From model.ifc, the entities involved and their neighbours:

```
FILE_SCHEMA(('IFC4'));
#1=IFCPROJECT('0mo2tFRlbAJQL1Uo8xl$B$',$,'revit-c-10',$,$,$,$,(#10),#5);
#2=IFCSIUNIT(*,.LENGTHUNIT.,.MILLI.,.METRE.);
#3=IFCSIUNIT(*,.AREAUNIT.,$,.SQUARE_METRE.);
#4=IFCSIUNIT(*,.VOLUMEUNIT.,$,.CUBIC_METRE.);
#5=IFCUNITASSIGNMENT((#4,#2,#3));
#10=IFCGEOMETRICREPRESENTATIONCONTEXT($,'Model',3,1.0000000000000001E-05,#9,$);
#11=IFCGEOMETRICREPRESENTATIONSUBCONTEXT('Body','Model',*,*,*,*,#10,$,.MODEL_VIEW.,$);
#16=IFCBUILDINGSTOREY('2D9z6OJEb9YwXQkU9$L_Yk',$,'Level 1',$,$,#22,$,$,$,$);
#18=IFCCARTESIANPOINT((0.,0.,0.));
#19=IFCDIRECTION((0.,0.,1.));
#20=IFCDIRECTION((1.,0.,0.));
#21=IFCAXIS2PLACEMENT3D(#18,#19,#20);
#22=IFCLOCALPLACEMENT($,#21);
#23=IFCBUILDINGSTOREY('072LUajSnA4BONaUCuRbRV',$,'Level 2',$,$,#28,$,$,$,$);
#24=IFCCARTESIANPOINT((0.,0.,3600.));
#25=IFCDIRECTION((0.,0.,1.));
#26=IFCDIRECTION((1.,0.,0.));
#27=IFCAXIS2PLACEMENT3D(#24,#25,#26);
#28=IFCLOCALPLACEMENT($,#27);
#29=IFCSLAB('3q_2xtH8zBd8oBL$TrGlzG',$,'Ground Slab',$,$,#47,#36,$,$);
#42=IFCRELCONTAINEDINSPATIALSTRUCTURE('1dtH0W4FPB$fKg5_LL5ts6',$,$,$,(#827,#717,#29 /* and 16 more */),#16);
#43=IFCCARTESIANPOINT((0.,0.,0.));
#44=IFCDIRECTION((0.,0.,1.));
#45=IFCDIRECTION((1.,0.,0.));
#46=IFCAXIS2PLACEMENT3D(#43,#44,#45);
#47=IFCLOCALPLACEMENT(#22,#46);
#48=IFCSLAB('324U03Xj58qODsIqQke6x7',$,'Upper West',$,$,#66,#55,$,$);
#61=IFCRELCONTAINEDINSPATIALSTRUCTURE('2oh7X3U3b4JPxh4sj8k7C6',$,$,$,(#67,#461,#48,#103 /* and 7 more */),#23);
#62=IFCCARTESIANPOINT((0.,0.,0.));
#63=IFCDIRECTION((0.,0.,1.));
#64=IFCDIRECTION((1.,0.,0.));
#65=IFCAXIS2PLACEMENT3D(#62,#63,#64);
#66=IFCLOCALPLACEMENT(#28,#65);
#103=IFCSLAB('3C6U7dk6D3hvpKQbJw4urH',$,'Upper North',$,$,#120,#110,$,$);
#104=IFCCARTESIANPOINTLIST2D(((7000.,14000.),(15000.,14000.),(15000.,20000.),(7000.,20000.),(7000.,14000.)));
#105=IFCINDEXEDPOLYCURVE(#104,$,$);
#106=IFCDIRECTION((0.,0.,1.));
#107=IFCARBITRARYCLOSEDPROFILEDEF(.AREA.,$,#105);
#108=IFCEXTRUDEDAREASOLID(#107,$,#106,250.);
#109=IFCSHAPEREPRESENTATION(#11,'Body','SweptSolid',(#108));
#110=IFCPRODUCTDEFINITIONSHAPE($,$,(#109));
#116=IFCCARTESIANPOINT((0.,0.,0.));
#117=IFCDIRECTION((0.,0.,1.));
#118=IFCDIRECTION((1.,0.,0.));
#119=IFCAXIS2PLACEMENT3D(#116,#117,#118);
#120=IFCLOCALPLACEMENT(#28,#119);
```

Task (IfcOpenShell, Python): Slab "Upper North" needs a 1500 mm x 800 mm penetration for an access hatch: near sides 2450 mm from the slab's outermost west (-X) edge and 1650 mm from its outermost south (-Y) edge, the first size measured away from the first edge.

```python
import numpy as np
import ifcopenshell
import ifcopenshell.api.feature
import ifcopenshell.api.geometry
import ifcopenshell.api.root
import ifcopenshell.geom
import ifcopenshell.util.placement
import ifcopenshell.util.representation
import ifcopenshell.util.shape
import ifcopenshell.util.unit

model = ifcopenshell.open("model.ifc")
unit_scale = ifcopenshell.util.unit.calculate_unit_scale(model)
settings = ifcopenshell.geom.settings()


def volume(element):
    """Net volume in cubic metres, openings subtracted."""
    shape = ifcopenshell.geom.create_shape(settings, element)
    return ifcopenshell.util.shape.get_volume(shape.geometry)


slab = model.by_id(103)
before = volume(slab)

# Extent in the slab's own axes, in metres. The edges named are its -X and -Y sides.
slab_shape = ifcopenshell.geom.create_shape(settings, slab)
vertices = ifcopenshell.util.shape.get_vertices(slab_shape.geometry)
x_min, y_min, bottom = vertices.min(axis=0)
top = vertices[:, 2].max()

opening = ifcopenshell.api.root.create_entity(model, ifc_class="IfcOpeningElement", name="Access hatch opening", predefined_type="OPENING")
context = ifcopenshell.util.representation.get_context(model, "Model", "Body", "MODEL_VIEW")
width, depth = 1.5, 0.8
outline = [(0.0, 0.0), (width, 0.0), (width, depth), (0.0, depth), (0.0, 0.0)]
# Overshoot both faces by 50 mm so the cut is clean.
shape = ifcopenshell.api.geometry.add_slab_representation(
    model, context=context, depth=top - bottom + 0.1, polyline=outline
)
ifcopenshell.api.geometry.assign_representation(model, product=opening, representation=shape)

matrix = ifcopenshell.util.placement.get_local_placement(slab.ObjectPlacement)
matrix[:, 3] = matrix @ np.append(np.array([x_min + 2.45, y_min + 1.65, bottom - 0.05]) / unit_scale, 1.0)
ifcopenshell.api.geometry.edit_object_placement(model, product=opening, matrix=matrix, is_si=False)
ifcopenshell.api.feature.add_feature(model, feature=opening, element=slab)

after = volume(slab)

print(f"slab volume {before:.3f} -> {after:.3f} m3")

model.write("model_updated.ifc")
```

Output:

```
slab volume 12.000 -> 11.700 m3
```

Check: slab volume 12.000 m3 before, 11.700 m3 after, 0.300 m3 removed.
